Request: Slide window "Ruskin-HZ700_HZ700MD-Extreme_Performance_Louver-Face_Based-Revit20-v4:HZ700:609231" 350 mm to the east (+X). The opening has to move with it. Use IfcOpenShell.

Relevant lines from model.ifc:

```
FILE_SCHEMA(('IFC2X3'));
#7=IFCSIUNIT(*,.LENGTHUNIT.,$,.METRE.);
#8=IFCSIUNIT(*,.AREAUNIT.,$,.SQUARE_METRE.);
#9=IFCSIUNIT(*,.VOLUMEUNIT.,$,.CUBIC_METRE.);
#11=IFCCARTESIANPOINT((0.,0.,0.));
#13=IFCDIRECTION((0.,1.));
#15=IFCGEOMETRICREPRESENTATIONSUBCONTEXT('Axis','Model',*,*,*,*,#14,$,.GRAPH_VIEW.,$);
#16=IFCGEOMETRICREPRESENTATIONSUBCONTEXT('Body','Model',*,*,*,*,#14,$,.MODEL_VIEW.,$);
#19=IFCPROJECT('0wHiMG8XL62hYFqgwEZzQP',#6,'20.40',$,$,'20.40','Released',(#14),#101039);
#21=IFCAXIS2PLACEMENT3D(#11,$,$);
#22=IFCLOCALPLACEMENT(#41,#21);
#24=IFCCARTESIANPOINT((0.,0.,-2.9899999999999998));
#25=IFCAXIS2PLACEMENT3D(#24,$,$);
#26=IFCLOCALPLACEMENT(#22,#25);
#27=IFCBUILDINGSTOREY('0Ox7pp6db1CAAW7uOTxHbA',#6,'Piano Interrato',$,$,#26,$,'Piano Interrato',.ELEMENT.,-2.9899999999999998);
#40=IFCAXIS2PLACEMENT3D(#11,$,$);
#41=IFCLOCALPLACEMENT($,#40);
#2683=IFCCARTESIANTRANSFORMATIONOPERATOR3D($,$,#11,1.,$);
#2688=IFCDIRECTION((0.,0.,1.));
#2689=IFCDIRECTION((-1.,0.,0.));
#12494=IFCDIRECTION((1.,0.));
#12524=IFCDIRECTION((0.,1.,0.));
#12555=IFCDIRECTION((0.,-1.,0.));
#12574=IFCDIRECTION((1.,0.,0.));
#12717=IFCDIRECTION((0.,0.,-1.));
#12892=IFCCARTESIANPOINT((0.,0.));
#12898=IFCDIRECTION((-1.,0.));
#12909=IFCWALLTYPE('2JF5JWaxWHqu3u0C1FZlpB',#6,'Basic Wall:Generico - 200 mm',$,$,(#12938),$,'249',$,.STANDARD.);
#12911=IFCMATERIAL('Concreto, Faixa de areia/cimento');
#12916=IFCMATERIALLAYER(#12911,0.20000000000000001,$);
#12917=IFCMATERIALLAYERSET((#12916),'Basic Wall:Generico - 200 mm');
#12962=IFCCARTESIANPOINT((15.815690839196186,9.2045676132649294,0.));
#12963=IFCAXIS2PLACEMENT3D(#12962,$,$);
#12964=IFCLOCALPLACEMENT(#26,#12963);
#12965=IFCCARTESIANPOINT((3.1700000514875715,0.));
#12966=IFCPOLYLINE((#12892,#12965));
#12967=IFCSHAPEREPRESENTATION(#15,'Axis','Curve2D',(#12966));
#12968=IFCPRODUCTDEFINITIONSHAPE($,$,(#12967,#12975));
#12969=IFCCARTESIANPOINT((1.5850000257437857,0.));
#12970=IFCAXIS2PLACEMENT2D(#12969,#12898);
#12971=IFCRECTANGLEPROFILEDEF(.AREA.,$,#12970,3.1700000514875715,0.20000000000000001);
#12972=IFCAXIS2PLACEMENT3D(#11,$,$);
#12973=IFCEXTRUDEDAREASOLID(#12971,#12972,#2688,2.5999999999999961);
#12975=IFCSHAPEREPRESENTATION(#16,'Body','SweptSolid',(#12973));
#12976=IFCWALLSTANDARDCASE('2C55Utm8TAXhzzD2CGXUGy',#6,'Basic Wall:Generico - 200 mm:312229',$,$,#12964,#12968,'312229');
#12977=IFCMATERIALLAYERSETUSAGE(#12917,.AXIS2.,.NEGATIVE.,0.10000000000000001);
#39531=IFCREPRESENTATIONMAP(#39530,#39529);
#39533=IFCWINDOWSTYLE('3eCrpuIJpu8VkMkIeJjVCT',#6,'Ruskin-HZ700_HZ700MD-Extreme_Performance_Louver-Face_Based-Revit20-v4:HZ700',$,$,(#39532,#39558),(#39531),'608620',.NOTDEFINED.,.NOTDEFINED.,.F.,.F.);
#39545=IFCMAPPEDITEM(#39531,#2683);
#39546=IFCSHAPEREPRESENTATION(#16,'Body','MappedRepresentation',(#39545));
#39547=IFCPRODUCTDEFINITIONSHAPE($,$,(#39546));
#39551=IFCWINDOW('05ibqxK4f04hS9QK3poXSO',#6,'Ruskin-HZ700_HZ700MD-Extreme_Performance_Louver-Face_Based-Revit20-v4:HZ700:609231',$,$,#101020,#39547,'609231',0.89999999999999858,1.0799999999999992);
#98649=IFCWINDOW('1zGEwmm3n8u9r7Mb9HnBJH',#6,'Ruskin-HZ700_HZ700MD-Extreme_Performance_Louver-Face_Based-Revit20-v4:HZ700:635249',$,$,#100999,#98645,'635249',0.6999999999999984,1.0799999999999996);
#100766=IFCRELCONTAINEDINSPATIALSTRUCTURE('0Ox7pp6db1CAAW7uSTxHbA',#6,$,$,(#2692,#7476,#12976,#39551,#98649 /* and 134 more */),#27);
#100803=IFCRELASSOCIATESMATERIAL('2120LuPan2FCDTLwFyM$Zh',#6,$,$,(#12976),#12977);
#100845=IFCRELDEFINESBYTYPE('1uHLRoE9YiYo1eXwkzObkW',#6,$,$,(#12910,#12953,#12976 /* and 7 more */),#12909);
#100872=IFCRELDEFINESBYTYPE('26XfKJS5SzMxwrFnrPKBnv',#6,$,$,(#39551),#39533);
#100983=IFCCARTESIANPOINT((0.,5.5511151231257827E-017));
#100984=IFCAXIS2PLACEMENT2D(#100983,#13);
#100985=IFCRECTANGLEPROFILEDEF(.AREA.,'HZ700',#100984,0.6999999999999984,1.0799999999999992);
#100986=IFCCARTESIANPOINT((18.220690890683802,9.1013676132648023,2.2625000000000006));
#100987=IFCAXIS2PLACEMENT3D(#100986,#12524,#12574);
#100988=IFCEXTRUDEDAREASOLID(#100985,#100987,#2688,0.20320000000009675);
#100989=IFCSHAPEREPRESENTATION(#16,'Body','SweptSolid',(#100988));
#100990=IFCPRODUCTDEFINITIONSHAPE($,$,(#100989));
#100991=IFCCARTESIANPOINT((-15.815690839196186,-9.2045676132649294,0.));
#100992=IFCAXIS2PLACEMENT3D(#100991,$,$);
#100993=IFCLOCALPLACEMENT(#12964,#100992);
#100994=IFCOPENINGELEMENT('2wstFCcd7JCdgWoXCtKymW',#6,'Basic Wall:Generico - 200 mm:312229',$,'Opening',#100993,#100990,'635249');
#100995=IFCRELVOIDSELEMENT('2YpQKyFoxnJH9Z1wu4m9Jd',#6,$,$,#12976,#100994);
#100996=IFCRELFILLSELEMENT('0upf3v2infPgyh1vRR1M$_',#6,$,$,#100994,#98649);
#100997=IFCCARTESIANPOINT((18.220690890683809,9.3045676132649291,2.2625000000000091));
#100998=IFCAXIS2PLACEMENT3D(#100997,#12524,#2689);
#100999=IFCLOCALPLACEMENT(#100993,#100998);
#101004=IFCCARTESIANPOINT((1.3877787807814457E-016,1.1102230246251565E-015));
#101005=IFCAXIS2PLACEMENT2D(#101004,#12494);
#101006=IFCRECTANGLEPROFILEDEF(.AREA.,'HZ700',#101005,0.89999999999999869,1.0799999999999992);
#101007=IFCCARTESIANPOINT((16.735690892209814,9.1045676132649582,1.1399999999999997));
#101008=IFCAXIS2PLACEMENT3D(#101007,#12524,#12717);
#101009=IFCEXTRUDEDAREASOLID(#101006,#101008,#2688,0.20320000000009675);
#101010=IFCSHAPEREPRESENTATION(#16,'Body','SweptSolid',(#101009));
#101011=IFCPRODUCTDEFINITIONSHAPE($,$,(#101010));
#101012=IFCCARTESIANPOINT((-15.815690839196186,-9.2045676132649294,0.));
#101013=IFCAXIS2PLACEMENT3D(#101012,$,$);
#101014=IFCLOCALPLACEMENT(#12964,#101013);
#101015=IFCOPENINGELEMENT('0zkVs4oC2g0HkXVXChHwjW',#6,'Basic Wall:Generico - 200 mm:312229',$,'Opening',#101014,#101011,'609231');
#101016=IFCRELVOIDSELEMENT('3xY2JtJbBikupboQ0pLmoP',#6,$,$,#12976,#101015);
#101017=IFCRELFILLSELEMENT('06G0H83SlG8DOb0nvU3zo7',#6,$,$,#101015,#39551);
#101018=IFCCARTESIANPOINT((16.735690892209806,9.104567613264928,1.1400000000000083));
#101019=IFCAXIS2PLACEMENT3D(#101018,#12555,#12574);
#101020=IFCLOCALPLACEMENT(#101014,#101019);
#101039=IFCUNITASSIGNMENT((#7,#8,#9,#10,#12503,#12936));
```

```python
import ifcopenshell
import ifcopenshell.api.geometry
import ifcopenshell.util.placement
import ifcopenshell.util.unit

model = ifcopenshell.open("model.ifc")
unit_scale = ifcopenshell.util.unit.calculate_unit_scale(model)

window = model.by_guid("05ibqxK4f04hS9QK3poXSO")
opening = window.FillsVoids[0].RelatingOpeningElement
wall = opening.VoidsElements[0].RelatingBuildingElement

wall_matrix = ifcopenshell.util.placement.get_local_placement(wall.ObjectPlacement)
shift = wall_matrix[:3, 0] * 0.35 / unit_scale
before = ifcopenshell.util.placement.get_local_placement(window.ObjectPlacement)[:3, 3].copy()

# The window is placed relative to its opening, so it follows when the opening moves.
matrix = ifcopenshell.util.placement.get_local_placement(opening.ObjectPlacement)
matrix[:3, 3] += shift
ifcopenshell.api.geometry.edit_object_placement(
    model, product=opening, matrix=matrix, is_si=False, should_transform_children=True
)

after = ifcopenshell.util.placement.get_local_placement(window.ObjectPlacement)[:3, 3]
print("window moved by", (after - before).round(3) + 0.0)

model.write("model_updated.ifc")
```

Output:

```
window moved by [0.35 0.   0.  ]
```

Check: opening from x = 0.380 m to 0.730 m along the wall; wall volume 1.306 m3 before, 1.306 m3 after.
